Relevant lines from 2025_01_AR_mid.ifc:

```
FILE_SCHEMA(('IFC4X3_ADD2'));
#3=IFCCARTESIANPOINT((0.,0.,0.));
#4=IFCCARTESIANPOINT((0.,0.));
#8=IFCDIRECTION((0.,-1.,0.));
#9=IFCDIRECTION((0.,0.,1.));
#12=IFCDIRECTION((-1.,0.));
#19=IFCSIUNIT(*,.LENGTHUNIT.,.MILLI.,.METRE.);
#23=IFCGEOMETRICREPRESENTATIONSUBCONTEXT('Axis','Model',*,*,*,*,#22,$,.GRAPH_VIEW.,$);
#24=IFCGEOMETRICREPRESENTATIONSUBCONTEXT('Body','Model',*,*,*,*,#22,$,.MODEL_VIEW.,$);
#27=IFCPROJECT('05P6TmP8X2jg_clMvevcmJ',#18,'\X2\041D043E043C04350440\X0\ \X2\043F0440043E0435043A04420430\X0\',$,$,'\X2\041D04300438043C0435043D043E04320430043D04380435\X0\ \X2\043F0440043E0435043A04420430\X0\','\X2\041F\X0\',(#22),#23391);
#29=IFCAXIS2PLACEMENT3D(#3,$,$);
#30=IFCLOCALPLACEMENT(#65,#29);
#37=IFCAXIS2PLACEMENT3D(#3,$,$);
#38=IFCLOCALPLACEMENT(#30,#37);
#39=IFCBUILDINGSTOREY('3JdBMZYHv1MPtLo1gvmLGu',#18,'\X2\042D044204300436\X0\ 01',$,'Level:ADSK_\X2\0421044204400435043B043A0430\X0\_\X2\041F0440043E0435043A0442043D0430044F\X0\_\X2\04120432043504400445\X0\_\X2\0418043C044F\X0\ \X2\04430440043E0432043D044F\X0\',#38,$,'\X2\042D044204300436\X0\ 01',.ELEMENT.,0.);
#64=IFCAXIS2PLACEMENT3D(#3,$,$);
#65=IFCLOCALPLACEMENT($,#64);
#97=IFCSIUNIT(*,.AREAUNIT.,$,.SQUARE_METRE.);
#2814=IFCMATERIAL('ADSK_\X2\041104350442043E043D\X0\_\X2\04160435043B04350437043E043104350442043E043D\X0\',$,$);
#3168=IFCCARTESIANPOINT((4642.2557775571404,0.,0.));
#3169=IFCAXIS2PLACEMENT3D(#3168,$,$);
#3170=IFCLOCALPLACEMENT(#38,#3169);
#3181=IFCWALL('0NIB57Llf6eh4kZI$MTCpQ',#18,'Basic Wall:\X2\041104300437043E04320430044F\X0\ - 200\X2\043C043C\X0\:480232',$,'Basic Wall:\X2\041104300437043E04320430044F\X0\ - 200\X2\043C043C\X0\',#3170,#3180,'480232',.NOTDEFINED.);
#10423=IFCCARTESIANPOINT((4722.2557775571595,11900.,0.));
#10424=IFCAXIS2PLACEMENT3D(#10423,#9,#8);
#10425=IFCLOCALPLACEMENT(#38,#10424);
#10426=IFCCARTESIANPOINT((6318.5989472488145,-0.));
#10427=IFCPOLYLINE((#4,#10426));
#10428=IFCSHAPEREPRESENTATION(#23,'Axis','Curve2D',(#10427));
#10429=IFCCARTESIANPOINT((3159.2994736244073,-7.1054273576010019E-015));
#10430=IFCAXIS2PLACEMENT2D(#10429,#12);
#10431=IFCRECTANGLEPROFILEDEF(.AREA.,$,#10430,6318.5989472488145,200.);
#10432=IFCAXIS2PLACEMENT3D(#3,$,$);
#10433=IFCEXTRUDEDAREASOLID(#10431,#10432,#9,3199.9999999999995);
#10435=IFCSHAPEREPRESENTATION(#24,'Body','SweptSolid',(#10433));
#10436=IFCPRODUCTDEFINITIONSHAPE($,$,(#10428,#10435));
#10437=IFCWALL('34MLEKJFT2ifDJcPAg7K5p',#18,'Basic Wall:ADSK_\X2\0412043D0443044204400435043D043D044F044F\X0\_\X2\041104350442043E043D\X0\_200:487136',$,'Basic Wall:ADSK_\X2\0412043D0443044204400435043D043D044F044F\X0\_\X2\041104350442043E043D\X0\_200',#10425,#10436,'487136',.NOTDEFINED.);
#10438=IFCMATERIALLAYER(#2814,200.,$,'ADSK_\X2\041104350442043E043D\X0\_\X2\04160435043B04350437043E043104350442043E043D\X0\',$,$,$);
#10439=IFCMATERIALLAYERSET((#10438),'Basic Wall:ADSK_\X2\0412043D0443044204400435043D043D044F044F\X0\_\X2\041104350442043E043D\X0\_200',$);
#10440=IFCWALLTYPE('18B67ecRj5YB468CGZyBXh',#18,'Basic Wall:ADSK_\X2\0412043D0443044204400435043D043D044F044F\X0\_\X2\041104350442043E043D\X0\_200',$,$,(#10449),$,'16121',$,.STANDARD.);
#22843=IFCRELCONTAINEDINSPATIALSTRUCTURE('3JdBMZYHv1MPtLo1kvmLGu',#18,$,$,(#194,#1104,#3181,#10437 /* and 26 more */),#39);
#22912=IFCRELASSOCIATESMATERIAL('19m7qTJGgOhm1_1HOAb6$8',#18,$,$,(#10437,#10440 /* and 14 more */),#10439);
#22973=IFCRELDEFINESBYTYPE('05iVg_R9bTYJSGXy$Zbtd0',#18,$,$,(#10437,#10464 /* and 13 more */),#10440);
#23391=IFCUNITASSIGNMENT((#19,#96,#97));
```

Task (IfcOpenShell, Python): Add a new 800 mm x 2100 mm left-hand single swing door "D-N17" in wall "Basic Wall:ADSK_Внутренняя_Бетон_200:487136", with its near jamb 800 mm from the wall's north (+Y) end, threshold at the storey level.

```python
import numpy as np
import ifcopenshell
import ifcopenshell.api.feature
import ifcopenshell.api.geometry
import ifcopenshell.api.root
import ifcopenshell.api.spatial
import ifcopenshell.geom
import ifcopenshell.util.element
import ifcopenshell.util.placement
import ifcopenshell.util.representation
import ifcopenshell.util.shape
import ifcopenshell.util.unit

model = ifcopenshell.open("2025_01_AR_mid.ifc")
unit_scale = ifcopenshell.util.unit.calculate_unit_scale(model)
settings = ifcopenshell.geom.settings()


def volume(element):
    """Net volume in cubic metres, openings subtracted."""
    shape = ifcopenshell.geom.create_shape(settings, element)
    return ifcopenshell.util.shape.get_volume(shape.geometry)


wall = model.by_id(10437)
storey = ifcopenshell.util.element.get_container(wall, ifc_class="IfcBuildingStorey")
context = ifcopenshell.util.representation.get_context(model, "Model", "Body", "MODEL_VIEW")
before = volume(wall)

width, height, from_end, sill = 0.8, 2.1, 0.8, 0.0  # metres

# The wall runs along its own X axis, and the end named is its -X end.
wall_shape = ifcopenshell.geom.create_shape(settings, wall)
x, y, z = ifcopenshell.util.shape.get_vertices(wall_shape.geometry).T
start = x.min() + from_end
face, thickness = float(y.min()), float(y.max() - y.min())
wall_matrix = ifcopenshell.util.placement.get_local_placement(wall.ObjectPlacement)
level = ifcopenshell.util.placement.get_local_placement(storey.ObjectPlacement)[2, 3]


def in_wall(x, y):
    """Placement at x, y metres in the wall's axes, at sill height."""
    matrix = wall_matrix.copy()
    matrix[:, 3] = wall_matrix @ np.array([x / unit_scale, y / unit_scale, 0.0, 1.0])
    matrix[2, 3] = level + sill / unit_scale
    return matrix


# Opening: a box that overshoots both wall faces by 50 mm.
opening = ifcopenshell.api.root.create_entity(model, ifc_class="IfcOpeningElement", predefined_type="OPENING")
box = ifcopenshell.api.geometry.add_wall_representation(
    model, context=context, length=width, height=height, thickness=thickness + 0.1
)
ifcopenshell.api.geometry.assign_representation(model, product=opening, representation=box)
ifcopenshell.api.geometry.edit_object_placement(model, product=opening, matrix=in_wall(start, face - 0.05), is_si=False)
ifcopenshell.api.feature.add_feature(model, feature=opening, element=wall)

door = ifcopenshell.api.root.create_entity(model, ifc_class="IfcDoor", name="D-N17", predefined_type="DOOR")
door.OverallWidth, door.OverallHeight = width / unit_scale, height / unit_scale
door.OperationType = "SINGLE_SWING_LEFT"
body = ifcopenshell.api.geometry.add_door_representation(
    model,
    context=context,
    overall_width=door.OverallWidth,
    overall_height=door.OverallHeight,
    operation_type="SINGLE_SWING_LEFT",
    lining_properties={"LiningDepth": thickness / unit_scale, "ThresholdDepth": thickness / unit_scale},
)
ifcopenshell.api.geometry.assign_representation(model, product=door, representation=body)
ifcopenshell.api.spatial.assign_container(model, products=[door], relating_structure=storey)
ifcopenshell.api.feature.add_filling(model, opening=opening, element=door)

# The lining spans the wall, so the door starts at the wall face.
ifcopenshell.api.geometry.edit_object_placement(model, product=door, matrix=in_wall(start, face), is_si=False)

after = volume(wall)

print(f"wall volume {before:.3f} -> {after:.3f} m3")

model.write("2025_01_AR_mid-out.ifc")
```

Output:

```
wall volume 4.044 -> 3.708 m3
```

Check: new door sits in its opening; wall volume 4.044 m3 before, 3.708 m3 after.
